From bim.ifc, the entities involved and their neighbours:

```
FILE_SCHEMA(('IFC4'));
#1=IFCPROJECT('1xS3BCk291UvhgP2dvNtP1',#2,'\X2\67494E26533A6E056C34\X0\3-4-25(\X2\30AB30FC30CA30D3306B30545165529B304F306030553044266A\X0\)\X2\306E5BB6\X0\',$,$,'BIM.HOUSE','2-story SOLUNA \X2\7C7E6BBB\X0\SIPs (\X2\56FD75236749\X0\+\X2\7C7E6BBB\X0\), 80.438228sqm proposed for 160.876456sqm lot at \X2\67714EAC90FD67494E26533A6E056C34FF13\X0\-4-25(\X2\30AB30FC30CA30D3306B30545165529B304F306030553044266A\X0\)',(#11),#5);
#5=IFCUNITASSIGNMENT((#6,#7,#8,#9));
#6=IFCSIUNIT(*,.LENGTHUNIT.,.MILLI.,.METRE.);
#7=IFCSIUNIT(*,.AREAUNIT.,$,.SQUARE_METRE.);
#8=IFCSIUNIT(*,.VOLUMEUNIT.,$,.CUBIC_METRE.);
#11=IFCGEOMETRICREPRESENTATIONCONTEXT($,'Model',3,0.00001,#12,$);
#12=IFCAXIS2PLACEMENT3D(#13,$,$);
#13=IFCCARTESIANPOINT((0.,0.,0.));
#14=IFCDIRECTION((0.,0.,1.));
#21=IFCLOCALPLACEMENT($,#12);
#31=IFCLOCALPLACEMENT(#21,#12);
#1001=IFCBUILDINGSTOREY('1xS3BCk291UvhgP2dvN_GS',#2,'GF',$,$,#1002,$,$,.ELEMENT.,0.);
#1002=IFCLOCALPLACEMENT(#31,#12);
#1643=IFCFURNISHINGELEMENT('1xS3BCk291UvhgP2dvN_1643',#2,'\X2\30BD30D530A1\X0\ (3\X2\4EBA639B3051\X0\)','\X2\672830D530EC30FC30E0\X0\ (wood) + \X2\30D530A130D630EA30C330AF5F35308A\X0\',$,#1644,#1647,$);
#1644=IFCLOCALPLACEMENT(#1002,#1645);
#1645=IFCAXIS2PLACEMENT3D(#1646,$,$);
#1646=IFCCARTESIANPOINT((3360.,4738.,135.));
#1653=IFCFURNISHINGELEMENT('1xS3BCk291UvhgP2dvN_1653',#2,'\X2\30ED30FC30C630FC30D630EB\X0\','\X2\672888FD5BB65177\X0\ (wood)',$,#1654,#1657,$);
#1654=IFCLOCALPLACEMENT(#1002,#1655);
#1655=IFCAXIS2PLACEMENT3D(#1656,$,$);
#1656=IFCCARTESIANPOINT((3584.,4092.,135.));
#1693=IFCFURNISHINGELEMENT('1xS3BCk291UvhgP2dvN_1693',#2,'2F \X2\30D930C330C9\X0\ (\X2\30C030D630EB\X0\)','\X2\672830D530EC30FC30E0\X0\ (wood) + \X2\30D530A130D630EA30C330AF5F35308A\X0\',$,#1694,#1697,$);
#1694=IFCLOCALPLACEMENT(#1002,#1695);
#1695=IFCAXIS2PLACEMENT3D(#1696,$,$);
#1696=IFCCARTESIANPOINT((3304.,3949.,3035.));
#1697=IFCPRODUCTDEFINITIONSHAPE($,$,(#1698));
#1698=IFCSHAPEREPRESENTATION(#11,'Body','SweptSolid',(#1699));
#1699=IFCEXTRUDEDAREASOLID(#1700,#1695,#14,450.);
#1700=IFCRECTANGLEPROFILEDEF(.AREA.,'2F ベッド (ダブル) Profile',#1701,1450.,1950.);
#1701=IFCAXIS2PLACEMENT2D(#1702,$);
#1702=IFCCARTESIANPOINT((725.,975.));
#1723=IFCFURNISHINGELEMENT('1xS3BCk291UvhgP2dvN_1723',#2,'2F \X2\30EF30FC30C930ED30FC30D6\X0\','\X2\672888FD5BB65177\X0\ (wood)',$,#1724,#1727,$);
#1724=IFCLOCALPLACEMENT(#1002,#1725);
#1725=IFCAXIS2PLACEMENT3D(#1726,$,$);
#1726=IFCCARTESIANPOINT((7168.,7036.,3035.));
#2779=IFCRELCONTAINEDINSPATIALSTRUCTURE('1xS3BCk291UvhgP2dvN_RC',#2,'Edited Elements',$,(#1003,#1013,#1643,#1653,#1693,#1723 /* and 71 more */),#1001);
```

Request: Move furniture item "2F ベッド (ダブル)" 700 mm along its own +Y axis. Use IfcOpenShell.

```python
import ifcopenshell
import ifcopenshell.api.geometry
import ifcopenshell.util.placement
import ifcopenshell.util.unit

model = ifcopenshell.open("bim.ifc")
unit_scale = ifcopenshell.util.unit.calculate_unit_scale(model)

item = model.by_guid("1xS3BCk291UvhgP2dvN_1693")
matrix = ifcopenshell.util.placement.get_local_placement(item.ObjectPlacement)
matrix[:3, 3] += matrix[:3, 1] * 0.7 / unit_scale
ifcopenshell.api.geometry.edit_object_placement(model, product=item, matrix=matrix, is_si=False)

print(ifcopenshell.util.placement.get_local_placement(item.ObjectPlacement).round(3) + 0.0)

model.write("bim-out.ifc")
```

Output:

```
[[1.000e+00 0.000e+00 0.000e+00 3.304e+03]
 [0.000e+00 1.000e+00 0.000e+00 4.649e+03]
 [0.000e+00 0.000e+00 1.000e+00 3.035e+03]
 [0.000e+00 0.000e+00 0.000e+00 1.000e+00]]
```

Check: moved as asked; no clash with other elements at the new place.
